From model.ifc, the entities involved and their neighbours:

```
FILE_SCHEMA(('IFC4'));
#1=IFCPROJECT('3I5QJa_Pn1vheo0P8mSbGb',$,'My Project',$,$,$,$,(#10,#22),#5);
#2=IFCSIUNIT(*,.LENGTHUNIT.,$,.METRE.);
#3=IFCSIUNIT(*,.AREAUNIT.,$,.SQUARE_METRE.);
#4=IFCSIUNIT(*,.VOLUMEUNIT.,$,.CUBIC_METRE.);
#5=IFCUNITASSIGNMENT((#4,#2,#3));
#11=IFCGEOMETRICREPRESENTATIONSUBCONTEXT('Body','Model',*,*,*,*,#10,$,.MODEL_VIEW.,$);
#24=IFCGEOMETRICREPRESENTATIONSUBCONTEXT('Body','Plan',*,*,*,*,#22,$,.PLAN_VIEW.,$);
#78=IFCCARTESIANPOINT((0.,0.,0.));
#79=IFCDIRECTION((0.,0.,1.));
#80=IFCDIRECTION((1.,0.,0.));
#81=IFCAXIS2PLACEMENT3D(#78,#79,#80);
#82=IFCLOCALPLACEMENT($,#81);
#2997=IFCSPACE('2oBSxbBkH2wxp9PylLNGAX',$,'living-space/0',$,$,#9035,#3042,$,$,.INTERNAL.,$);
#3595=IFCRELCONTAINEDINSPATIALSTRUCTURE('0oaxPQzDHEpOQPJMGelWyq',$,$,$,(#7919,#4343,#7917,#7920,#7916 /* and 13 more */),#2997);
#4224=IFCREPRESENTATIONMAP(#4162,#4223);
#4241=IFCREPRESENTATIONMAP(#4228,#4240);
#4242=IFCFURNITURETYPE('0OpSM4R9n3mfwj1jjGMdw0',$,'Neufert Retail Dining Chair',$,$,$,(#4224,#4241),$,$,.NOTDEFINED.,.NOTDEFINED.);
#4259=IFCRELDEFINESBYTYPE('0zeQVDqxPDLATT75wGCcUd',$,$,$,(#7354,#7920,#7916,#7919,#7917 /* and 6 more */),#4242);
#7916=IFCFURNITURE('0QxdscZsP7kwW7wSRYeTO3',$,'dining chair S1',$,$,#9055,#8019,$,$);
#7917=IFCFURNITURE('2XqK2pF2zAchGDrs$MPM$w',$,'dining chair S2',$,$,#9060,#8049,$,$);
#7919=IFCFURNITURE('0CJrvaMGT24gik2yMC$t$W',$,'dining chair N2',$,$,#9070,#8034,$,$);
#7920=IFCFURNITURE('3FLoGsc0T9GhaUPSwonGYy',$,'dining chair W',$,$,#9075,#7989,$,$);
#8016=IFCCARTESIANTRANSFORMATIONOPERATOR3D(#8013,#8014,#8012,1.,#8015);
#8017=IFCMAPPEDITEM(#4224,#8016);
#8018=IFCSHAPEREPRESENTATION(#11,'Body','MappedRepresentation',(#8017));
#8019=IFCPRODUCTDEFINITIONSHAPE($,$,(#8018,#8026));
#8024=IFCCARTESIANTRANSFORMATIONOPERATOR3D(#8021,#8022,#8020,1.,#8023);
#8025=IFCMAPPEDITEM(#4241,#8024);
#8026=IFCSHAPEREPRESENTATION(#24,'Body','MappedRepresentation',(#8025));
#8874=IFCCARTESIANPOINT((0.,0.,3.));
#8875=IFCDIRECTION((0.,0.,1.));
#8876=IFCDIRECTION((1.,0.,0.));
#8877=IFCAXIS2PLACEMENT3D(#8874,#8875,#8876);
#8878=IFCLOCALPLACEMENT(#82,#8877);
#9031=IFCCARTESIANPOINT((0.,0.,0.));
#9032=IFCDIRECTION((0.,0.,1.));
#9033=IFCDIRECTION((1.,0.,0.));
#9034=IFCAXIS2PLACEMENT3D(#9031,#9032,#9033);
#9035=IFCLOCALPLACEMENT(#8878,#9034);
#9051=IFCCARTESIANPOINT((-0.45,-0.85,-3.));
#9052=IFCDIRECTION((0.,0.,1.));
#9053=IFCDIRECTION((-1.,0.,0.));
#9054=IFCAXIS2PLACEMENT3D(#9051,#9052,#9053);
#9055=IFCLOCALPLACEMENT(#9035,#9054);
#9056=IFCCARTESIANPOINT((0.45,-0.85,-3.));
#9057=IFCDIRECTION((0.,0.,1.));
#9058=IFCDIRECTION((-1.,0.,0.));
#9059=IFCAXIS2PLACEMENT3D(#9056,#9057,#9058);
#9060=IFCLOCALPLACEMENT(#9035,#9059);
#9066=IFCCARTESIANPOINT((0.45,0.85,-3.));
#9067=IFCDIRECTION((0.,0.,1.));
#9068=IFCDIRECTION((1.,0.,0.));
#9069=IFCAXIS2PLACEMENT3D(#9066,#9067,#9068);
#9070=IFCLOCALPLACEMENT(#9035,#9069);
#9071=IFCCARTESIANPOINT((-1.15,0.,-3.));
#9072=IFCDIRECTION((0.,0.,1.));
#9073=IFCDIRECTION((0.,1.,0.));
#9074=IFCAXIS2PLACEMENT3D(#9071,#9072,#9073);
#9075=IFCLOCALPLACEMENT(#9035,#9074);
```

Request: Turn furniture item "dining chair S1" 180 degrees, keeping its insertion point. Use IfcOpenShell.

```python
import ifcopenshell
import ifcopenshell.api.geometry
import ifcopenshell.util.placement

model = ifcopenshell.open("model.ifc")

item = model.by_id(7916)
matrix = ifcopenshell.util.placement.get_local_placement(item.ObjectPlacement)
matrix = matrix @ ifcopenshell.util.placement.rotation(180, "Z")
ifcopenshell.api.geometry.edit_object_placement(model, product=item, matrix=matrix, is_si=False)

print(ifcopenshell.util.placement.get_local_placement(item.ObjectPlacement).round(3) + 0.0)

model.write("model_edited.ifc")
```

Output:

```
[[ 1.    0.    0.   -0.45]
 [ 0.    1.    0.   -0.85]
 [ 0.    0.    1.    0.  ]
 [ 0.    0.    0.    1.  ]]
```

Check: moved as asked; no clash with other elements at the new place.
